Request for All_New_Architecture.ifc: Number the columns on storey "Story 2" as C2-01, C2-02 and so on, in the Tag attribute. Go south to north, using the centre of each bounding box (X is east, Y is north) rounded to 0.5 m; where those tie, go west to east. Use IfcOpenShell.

First a look at what the model holds.

```python
import ifcopenshell
import ifcopenshell.util.element
import ifcopenshell.util.placement

model = ifcopenshell.open("All_New_Architecture.ifc")
print(model.schema)
storey = next(s for s in model.by_type("IfcBuildingStorey") if s.Name == "Story 2")
columns = [e for e in ifcopenshell.util.element.get_decomposition(storey) if e.is_a("IfcColumn")]
for e in sorted(columns, key=lambda e: e.id()):
    origin = ifcopenshell.util.placement.get_local_placement(e.ObjectPlacement)[:3, 3]
    print(e.id(), e.Tag, e.Name, origin.round(2) + 0.0, sep=" | ")
```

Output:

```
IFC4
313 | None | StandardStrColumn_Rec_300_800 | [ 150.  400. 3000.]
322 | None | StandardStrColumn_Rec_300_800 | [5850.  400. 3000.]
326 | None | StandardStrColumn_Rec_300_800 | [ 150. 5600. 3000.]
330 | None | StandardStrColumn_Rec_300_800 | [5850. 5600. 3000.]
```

```python
import ifcopenshell
import ifcopenshell.geom
import ifcopenshell.util.element
import ifcopenshell.util.shape

model = ifcopenshell.open("All_New_Architecture.ifc")
settings = ifcopenshell.geom.settings()
settings.set("use-world-coords", True)


def centre(element):
    shape = ifcopenshell.geom.create_shape(settings, element)
    return ifcopenshell.util.shape.get_bbox_centroid(shape.geometry)


storey = next(s for s in model.by_type("IfcBuildingStorey") if s.Name == "Story 2")
columns = [e for e in ifcopenshell.util.element.get_decomposition(storey) if e.is_a("IfcColumn")]

# Insertion points can sit at a corner or the storey origin, so sort by the geometry (in metres).
centres = {e: centre(e) for e in columns}
columns.sort(key=lambda e: (round(centres[e][1] / 0.5), centres[e][0]))

for i, e in enumerate(columns, start=1):
    number = f"C2-{i:02d}"
    e.Tag = number
    print(e.id(), number)

model.write("All_New_Architecture-out.ifc")
```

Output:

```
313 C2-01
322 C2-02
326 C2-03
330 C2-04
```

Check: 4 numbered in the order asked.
